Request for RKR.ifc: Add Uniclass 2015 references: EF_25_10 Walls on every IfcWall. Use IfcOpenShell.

First a look at what the model holds.

```python
import ifcopenshell

model = ifcopenshell.open("RKR.ifc")
print(model.schema)
print("classifications:", [c.Name for c in model.by_type("IfcClassification")])
for ifc_class in ("IfcDoor", "IfcRoof", "IfcStair", "IfcWall", "IfcWindow"):
    print(ifc_class, len(model.by_type(ifc_class)))
```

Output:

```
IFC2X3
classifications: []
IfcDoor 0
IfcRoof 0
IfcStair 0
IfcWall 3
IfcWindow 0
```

```python
import ifcopenshell
import ifcopenshell.api.classification

model = ifcopenshell.open("RKR.ifc")

# IFC2X3 requires Source and Edition and has no link from the project to the system.
system = model.create_entity("IfcClassification", Source="NBS", Edition="2015", Name="Uniclass 2015")

codes = {
    "IfcWall": ("EF_25_10", "Walls"),
}
for ifc_class, (code, name) in codes.items():
    products = model.by_type(ifc_class)
    ifcopenshell.api.classification.add_reference(
        model, products=products, classification=system, identification=code, name=name
    )
    print(code, len(products))

model.write("RKR_edited.ifc")
```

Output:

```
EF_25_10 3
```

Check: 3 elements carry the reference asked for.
